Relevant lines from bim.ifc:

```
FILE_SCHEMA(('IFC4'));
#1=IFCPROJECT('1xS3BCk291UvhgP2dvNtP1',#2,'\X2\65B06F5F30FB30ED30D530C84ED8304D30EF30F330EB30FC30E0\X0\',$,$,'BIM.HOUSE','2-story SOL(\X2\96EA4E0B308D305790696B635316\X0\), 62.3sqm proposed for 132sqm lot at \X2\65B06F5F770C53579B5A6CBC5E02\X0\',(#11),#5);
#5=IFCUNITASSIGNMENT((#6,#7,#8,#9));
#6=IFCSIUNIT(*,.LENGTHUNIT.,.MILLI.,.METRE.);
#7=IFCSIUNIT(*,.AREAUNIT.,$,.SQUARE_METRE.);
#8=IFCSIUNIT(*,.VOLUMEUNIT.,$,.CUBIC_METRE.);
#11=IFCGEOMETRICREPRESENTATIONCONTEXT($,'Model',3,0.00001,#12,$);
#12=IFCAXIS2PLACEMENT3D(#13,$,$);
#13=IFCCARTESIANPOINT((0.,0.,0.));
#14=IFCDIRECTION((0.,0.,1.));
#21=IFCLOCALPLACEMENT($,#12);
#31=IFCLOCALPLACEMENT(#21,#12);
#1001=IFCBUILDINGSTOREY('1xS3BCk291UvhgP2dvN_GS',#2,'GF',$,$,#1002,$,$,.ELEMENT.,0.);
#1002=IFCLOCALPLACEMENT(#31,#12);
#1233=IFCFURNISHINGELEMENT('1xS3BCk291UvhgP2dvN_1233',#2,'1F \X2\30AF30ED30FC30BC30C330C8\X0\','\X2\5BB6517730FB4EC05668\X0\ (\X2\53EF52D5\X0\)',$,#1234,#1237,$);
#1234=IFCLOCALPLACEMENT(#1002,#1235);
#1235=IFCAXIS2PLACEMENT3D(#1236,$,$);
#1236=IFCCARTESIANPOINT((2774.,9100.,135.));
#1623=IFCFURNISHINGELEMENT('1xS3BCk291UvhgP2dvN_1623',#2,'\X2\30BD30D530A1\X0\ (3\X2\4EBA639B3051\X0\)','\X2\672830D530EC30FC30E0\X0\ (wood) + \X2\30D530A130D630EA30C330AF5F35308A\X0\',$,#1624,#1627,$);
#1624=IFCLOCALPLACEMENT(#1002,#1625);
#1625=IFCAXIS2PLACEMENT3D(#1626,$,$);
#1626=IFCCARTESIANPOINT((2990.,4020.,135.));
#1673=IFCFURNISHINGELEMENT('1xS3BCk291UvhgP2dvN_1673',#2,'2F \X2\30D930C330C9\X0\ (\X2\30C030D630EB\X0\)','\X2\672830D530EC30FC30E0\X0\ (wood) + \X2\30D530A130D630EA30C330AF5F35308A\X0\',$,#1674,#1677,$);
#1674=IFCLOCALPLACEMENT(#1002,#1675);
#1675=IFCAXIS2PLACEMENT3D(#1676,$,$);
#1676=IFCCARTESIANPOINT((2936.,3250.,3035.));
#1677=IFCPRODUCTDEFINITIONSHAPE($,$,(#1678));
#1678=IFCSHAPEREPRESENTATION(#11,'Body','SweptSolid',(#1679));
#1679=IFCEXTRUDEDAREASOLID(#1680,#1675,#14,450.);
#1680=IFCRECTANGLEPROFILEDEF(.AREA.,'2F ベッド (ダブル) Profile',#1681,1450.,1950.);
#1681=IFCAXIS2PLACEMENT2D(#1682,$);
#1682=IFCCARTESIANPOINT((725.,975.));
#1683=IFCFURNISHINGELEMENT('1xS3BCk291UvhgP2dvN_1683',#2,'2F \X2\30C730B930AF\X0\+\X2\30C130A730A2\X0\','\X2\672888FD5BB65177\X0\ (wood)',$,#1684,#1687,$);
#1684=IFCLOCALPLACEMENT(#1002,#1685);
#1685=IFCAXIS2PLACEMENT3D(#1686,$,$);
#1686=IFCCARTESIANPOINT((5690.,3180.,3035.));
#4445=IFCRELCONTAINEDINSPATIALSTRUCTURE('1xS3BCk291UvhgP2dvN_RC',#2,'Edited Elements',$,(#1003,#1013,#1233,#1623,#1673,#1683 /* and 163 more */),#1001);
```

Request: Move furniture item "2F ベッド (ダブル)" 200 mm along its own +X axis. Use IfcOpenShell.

```python
import ifcopenshell
import ifcopenshell.api.geometry
import ifcopenshell.util.placement
import ifcopenshell.util.unit

model = ifcopenshell.open("bim.ifc")
unit_scale = ifcopenshell.util.unit.calculate_unit_scale(model)

item = model.by_id(1673)
matrix = ifcopenshell.util.placement.get_local_placement(item.ObjectPlacement)
matrix[:3, 3] += matrix[:3, 0] * 0.2 / unit_scale
ifcopenshell.api.geometry.edit_object_placement(model, product=item, matrix=matrix, is_si=False)

print(ifcopenshell.util.placement.get_local_placement(item.ObjectPlacement).round(3) + 0.0)

model.write("bim_edited.ifc")
```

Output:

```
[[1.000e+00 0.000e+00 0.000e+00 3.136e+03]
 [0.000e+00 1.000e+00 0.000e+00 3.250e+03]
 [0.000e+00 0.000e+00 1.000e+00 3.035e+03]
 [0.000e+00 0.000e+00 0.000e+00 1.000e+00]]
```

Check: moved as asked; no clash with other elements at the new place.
